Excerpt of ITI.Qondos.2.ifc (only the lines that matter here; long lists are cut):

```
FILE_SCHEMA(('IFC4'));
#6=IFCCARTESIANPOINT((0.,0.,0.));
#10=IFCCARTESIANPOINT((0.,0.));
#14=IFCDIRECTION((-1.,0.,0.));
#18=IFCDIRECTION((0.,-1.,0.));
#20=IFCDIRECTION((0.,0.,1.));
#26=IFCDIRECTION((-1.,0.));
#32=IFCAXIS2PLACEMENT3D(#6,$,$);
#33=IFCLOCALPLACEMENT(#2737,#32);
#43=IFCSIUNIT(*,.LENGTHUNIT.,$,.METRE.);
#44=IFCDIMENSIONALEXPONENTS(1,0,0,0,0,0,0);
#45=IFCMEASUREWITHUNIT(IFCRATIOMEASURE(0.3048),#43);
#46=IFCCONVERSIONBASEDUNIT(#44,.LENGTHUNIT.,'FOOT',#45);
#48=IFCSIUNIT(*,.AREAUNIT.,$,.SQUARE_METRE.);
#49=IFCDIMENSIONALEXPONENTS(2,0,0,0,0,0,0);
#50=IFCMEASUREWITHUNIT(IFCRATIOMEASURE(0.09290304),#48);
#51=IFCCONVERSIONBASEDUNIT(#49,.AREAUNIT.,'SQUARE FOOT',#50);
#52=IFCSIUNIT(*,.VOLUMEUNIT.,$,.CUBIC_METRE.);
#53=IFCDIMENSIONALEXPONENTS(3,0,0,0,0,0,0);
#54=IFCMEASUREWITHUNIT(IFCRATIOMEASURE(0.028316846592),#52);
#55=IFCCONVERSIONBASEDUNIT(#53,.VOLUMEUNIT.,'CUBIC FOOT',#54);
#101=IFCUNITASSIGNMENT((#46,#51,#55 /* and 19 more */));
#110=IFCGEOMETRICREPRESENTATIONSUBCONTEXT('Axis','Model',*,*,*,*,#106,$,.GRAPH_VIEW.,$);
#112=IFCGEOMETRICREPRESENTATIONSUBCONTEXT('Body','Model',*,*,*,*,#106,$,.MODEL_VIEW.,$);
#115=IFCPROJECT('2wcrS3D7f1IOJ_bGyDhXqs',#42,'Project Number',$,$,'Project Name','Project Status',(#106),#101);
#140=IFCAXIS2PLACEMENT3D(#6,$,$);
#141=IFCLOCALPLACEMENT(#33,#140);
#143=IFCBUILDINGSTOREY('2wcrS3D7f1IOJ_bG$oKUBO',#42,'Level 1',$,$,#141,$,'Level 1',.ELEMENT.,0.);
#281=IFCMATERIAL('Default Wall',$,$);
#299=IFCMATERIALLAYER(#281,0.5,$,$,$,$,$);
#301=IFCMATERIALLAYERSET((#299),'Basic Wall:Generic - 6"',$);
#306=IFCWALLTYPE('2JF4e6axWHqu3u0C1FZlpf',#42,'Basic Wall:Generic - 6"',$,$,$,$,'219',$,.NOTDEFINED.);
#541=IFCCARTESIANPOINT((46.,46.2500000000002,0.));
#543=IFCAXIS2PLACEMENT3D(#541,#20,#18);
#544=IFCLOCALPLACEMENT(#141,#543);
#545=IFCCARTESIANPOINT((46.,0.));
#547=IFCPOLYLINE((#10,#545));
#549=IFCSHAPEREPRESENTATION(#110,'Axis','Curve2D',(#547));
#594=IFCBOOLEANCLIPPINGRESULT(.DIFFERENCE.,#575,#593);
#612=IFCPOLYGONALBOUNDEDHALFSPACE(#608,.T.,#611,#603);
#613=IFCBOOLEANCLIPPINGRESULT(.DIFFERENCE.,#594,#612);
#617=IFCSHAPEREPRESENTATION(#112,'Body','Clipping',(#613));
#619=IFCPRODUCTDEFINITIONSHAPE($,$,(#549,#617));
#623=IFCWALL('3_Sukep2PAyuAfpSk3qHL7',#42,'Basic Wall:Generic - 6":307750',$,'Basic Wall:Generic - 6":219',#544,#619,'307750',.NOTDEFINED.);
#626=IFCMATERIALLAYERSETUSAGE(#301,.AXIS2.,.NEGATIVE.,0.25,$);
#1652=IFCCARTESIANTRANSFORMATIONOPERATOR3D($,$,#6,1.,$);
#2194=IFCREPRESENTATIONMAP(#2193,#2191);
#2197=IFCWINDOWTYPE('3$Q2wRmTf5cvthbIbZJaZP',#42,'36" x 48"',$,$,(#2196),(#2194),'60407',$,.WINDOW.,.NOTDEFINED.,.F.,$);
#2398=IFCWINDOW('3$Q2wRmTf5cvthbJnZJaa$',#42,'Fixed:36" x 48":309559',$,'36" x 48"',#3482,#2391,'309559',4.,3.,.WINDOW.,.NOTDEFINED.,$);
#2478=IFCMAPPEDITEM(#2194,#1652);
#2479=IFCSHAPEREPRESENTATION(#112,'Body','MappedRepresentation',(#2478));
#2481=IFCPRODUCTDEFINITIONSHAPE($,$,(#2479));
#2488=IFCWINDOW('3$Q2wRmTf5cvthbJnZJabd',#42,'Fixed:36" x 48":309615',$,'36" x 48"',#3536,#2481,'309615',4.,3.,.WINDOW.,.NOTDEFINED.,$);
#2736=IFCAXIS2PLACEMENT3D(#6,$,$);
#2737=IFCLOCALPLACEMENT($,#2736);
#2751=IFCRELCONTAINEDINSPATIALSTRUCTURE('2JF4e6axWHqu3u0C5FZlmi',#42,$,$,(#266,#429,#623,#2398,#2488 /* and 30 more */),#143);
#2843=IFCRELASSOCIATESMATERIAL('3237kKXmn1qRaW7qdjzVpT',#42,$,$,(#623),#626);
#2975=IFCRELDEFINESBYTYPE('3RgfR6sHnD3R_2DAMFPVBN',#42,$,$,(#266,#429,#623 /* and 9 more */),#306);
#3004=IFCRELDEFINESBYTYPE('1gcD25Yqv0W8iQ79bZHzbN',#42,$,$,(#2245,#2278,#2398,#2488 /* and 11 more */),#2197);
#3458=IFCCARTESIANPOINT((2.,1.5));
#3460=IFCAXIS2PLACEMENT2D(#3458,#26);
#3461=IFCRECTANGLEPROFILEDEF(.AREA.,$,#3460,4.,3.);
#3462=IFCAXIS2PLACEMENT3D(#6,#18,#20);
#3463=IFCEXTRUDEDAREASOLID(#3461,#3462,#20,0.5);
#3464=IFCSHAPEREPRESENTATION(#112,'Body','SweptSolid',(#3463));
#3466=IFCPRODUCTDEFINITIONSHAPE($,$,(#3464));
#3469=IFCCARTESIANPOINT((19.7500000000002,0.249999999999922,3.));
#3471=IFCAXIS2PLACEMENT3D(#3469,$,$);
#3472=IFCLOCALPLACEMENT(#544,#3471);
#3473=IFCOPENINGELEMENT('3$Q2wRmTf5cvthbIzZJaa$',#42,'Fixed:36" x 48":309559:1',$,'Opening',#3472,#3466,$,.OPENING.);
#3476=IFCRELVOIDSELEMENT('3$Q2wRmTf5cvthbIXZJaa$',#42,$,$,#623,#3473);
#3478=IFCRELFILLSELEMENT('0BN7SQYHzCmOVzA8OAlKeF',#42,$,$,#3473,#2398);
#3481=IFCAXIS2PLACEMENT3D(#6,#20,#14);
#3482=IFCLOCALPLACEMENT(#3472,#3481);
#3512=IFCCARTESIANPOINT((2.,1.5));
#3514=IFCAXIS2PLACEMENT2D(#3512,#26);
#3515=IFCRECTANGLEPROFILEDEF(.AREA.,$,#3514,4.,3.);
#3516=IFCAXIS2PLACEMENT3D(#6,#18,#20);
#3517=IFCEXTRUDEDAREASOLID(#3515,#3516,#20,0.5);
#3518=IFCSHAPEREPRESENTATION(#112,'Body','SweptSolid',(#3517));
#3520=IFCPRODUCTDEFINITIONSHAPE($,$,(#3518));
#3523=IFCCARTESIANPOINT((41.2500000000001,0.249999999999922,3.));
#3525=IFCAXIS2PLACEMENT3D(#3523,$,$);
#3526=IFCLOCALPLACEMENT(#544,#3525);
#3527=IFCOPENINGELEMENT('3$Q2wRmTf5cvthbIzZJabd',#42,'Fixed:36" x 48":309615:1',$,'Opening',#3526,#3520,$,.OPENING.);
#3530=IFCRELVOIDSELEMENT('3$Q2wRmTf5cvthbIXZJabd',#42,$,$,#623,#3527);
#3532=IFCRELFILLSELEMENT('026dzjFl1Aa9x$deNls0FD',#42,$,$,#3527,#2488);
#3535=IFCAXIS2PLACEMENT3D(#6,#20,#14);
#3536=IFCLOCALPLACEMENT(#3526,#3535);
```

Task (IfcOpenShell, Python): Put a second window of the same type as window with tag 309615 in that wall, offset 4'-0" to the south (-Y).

```python
import ifcopenshell
import ifcopenshell.api.feature
import ifcopenshell.api.geometry
import ifcopenshell.api.root
import ifcopenshell.geom
import ifcopenshell.util.element
import ifcopenshell.util.placement
import ifcopenshell.util.shape
import ifcopenshell.util.unit

model = ifcopenshell.open("ITI.Qondos.2.ifc")
unit_scale = ifcopenshell.util.unit.calculate_unit_scale(model)
settings = ifcopenshell.geom.settings()


def volume(element):
    """Net volume in cubic metres, openings subtracted."""
    shape = ifcopenshell.geom.create_shape(settings, element)
    return ifcopenshell.util.shape.get_volume(shape.geometry)


def reuse_history(source, copy):
    """copy_class also copies each property set's owner history, people and application; keep the originals."""
    for rel in copy.IsDefinedBy:
        if rel.is_a("IfcRelDefinesByProperties") and (history := rel.RelatingPropertyDefinition.OwnerHistory):
            rel.RelatingPropertyDefinition.OwnerHistory = source.OwnerHistory
            ifcopenshell.util.element.remove_deep2(model, history)


window = model.by_guid("3$Q2wRmTf5cvthbJnZJabd")
opening = window.FillsVoids[0].RelatingOpeningElement
wall = opening.VoidsElements[0].RelatingBuildingElement
before = volume(wall)
shift = ifcopenshell.util.placement.get_local_placement(wall.ObjectPlacement)[:3, 0] * 48 * 0.0254 / unit_scale

# copy_class copies the void relationship, type, container and properties, but no geometry.
new_opening = ifcopenshell.api.root.copy_class(model, product=opening)
new_opening.Representation = ifcopenshell.util.element.copy_deep(
    model, opening.Representation, exclude=["IfcGeometricRepresentationContext", "IfcRepresentationMap"]
)
new_opening.Name = 'Fixed:36" x 48"'
new_window = ifcopenshell.api.root.copy_class(model, product=window)
new_window.Representation = ifcopenshell.util.element.copy_deep(
    model, window.Representation, exclude=["IfcGeometricRepresentationContext", "IfcRepresentationMap"]
)
new_window.Name = 'Fixed:36" x 48"'
new_window.Tag = None
reuse_history(window, new_window)
ifcopenshell.api.feature.add_filling(model, opening=new_opening, element=new_window)

for old, new in ((opening, new_opening), (window, new_window)):
    matrix = ifcopenshell.util.placement.get_local_placement(old.ObjectPlacement)
    matrix[:3, 3] += shift
    ifcopenshell.api.geometry.edit_object_placement(model, product=new, matrix=matrix, is_si=False)

after = volume(wall)

print(f"wall volume {before:.3f} -> {after:.3f} m3")

model.write("ITI.Qondos.2_edited.ifc")
```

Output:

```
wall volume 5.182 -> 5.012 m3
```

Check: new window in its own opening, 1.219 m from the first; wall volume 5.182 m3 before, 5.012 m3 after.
